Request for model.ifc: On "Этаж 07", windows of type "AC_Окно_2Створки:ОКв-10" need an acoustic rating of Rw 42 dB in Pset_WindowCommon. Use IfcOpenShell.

First a look at what the model holds.

```python
import ifcopenshell
import ifcopenshell.util.element

model = ifcopenshell.open("model.ifc")
print(model.schema)
storey = next(s for s in model.by_type("IfcBuildingStorey") if s.Name == "Этаж 07")
windows = [e for e in ifcopenshell.util.element.get_decomposition(storey) if e.is_a("IfcWindow")]
seen = {}
for e in windows:
    element_type = ifcopenshell.util.element.get_type(e)
    key = (element_type.Name if element_type != e and element_type else None, ifcopenshell.util.element.get_pset(e, "Pset_WindowCommon", "AcousticRating"))
    seen[key] = seen.get(key, 0) + 1
for (name, value), count in sorted(seen.items(), key=str):
    print(count, "x", name, "|", value)
```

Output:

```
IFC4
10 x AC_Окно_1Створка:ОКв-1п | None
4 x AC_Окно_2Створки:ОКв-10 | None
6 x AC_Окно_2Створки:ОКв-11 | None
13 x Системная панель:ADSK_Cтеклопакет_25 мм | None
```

```python
import ifcopenshell
import ifcopenshell.api.pset
import ifcopenshell.util.element

model = ifcopenshell.open("model.ifc")

storey = next(s for s in model.by_type("IfcBuildingStorey") if s.Name == "Этаж 07")
windows = [e for e in ifcopenshell.util.element.get_decomposition(storey) if e.is_a("IfcWindow")]

count = 0
for e in windows:
    element_type = ifcopenshell.util.element.get_type(e)
    if element_type in (None, e) or element_type.Name != "AC_Окно_2Створки:ОКв-10":
        continue
    # add_pset returns the element's existing set when there is one.
    pset = ifcopenshell.api.pset.add_pset(model, product=e, name="Pset_WindowCommon")
    ifcopenshell.api.pset.edit_pset(model, pset=pset, properties={"AcousticRating": "Rw 42 dB"})
    count += 1

print(count, "windows updated")

model.write("model_rev.ifc")
```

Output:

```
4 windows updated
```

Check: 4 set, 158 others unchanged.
